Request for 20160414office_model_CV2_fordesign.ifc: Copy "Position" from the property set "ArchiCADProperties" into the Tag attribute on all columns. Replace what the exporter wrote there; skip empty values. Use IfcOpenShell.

First a look at what the model holds.

```python
import ifcopenshell
import ifcopenshell.util.element

model = ifcopenshell.open("20160414office_model_CV2_fordesign.ifc")
print(model.schema)
columns = model.by_type("IfcColumn")
print(len(columns), "columns")
for e in columns[:8]:
    source = ifcopenshell.util.element.get_pset(e, "ArchiCADProperties", "Position")
    target = e.Tag
    print(e.id(), repr(source), repr(target), sep=" | ")
```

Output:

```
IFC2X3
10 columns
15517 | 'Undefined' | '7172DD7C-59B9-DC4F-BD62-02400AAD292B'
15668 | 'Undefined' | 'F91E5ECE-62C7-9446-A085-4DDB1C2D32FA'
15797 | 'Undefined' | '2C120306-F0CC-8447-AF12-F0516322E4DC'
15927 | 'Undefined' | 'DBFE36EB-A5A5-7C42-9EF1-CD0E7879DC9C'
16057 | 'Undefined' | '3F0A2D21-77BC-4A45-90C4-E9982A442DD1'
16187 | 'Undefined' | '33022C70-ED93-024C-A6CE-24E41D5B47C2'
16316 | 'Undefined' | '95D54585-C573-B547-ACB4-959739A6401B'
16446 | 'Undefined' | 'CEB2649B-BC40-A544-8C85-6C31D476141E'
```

```python
import ifcopenshell
import ifcopenshell.util.element

model = ifcopenshell.open("20160414office_model_CV2_fordesign.ifc")

count = 0
for e in model.by_type("IfcColumn"):
    value = ifcopenshell.util.element.get_pset(e, "ArchiCADProperties", "Position")
    current = e.Tag
    if not value or not value.strip() or current == value:
        continue
    e.Tag = value
    count += 1

print(count, "columns updated")

model.write("20160414office_model_CV2_fordesign_updated.ifc")
```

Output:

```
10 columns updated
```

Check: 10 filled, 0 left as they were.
